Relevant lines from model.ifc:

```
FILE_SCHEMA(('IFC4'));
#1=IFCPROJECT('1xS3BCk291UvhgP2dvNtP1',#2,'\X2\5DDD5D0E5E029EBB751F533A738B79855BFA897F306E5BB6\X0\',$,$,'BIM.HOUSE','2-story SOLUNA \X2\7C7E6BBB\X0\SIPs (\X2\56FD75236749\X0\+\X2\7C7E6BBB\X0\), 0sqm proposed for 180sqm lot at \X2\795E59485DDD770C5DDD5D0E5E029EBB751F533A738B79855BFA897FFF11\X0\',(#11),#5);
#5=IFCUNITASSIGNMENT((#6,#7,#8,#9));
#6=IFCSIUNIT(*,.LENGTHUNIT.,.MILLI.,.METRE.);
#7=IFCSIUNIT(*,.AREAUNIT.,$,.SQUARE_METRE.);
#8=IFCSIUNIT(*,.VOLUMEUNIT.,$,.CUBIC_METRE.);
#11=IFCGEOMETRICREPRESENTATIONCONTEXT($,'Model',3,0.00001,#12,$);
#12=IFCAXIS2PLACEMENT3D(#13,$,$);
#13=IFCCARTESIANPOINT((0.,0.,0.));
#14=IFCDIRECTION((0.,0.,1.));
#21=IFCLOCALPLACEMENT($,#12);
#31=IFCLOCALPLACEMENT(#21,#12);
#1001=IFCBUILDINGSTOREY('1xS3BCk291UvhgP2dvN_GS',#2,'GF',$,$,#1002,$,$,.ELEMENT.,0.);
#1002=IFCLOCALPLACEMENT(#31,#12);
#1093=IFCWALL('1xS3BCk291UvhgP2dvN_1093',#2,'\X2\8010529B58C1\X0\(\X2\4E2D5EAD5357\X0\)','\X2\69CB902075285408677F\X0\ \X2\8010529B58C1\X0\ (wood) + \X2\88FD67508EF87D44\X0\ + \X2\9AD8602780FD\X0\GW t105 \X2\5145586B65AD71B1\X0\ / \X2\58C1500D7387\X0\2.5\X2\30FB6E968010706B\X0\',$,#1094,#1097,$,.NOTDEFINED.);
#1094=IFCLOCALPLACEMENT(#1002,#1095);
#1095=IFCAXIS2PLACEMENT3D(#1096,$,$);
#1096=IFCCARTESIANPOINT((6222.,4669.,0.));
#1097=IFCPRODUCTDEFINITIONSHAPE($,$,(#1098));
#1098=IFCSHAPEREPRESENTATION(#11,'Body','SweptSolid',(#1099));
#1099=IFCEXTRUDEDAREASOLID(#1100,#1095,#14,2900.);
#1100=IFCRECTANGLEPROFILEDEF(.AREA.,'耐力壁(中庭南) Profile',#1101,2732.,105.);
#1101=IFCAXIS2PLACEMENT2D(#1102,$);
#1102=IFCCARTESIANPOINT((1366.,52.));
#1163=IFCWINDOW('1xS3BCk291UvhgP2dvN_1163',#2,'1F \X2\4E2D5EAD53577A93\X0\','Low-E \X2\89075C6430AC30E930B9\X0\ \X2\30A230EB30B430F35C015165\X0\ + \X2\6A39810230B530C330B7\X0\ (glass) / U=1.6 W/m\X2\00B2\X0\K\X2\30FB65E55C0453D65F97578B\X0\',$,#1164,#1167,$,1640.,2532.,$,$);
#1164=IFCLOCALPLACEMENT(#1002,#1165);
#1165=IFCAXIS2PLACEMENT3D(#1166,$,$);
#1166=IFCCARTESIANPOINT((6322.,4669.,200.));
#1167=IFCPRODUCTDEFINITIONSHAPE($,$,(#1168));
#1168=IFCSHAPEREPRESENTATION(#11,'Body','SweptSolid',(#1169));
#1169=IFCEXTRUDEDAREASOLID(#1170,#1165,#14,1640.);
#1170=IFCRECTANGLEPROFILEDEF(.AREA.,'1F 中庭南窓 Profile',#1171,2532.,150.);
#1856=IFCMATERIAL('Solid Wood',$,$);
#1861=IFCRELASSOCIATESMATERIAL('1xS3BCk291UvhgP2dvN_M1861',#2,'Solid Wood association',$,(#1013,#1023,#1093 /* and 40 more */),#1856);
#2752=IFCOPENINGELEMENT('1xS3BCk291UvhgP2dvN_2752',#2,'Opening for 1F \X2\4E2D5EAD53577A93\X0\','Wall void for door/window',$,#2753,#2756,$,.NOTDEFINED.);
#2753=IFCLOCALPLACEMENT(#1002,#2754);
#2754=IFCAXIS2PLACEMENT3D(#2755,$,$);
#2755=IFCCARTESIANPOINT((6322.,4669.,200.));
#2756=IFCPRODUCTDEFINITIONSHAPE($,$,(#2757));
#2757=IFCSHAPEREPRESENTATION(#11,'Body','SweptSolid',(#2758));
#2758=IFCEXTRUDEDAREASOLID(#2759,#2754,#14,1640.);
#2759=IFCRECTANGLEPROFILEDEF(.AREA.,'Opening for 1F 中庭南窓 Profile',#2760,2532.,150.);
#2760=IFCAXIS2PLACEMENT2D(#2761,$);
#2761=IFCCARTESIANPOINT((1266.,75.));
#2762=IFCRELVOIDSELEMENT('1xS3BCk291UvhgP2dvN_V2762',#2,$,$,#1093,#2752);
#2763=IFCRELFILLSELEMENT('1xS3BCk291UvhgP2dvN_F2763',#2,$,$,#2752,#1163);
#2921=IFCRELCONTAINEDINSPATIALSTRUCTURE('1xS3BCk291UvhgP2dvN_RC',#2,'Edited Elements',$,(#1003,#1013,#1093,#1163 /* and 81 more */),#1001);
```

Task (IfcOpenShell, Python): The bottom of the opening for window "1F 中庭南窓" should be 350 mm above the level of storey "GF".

```python
import numpy as np
import ifcopenshell
import ifcopenshell.api.geometry
import ifcopenshell.geom
import ifcopenshell.util.element
import ifcopenshell.util.placement
import ifcopenshell.util.shape
import ifcopenshell.util.unit

model = ifcopenshell.open("model.ifc")
unit_scale = ifcopenshell.util.unit.calculate_unit_scale(model)

window = model.by_guid("1xS3BCk291UvhgP2dvN_1163")
opening = window.FillsVoids[0].RelatingOpeningElement
storey = ifcopenshell.util.element.get_container(window, ifc_class="IfcBuildingStorey")
level = ifcopenshell.util.placement.get_local_placement(storey.ObjectPlacement)[2, 3]

# The opening's origin need not be at the sill, so measure its lowest point.
shape = ifcopenshell.geom.create_shape(ifcopenshell.geom.settings(), opening)
bottom = ifcopenshell.util.shape.get_shape_bottom_elevation(shape, shape.geometry) / unit_scale
dz = level + 350.0 - bottom

shift = np.array([0.0, 0.0, dz])
# The window is not placed relative to its opening, so move both.
for product in (opening, window):
    matrix = ifcopenshell.util.placement.get_local_placement(product.ObjectPlacement)
    matrix[:3, 3] += shift
    ifcopenshell.api.geometry.edit_object_placement(model, product=product, matrix=matrix, is_si=False)

print(f"moved by {dz * unit_scale:+.3f} m")

model.write("model-out.ifc")
```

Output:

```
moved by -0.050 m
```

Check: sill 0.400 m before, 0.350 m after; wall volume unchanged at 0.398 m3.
